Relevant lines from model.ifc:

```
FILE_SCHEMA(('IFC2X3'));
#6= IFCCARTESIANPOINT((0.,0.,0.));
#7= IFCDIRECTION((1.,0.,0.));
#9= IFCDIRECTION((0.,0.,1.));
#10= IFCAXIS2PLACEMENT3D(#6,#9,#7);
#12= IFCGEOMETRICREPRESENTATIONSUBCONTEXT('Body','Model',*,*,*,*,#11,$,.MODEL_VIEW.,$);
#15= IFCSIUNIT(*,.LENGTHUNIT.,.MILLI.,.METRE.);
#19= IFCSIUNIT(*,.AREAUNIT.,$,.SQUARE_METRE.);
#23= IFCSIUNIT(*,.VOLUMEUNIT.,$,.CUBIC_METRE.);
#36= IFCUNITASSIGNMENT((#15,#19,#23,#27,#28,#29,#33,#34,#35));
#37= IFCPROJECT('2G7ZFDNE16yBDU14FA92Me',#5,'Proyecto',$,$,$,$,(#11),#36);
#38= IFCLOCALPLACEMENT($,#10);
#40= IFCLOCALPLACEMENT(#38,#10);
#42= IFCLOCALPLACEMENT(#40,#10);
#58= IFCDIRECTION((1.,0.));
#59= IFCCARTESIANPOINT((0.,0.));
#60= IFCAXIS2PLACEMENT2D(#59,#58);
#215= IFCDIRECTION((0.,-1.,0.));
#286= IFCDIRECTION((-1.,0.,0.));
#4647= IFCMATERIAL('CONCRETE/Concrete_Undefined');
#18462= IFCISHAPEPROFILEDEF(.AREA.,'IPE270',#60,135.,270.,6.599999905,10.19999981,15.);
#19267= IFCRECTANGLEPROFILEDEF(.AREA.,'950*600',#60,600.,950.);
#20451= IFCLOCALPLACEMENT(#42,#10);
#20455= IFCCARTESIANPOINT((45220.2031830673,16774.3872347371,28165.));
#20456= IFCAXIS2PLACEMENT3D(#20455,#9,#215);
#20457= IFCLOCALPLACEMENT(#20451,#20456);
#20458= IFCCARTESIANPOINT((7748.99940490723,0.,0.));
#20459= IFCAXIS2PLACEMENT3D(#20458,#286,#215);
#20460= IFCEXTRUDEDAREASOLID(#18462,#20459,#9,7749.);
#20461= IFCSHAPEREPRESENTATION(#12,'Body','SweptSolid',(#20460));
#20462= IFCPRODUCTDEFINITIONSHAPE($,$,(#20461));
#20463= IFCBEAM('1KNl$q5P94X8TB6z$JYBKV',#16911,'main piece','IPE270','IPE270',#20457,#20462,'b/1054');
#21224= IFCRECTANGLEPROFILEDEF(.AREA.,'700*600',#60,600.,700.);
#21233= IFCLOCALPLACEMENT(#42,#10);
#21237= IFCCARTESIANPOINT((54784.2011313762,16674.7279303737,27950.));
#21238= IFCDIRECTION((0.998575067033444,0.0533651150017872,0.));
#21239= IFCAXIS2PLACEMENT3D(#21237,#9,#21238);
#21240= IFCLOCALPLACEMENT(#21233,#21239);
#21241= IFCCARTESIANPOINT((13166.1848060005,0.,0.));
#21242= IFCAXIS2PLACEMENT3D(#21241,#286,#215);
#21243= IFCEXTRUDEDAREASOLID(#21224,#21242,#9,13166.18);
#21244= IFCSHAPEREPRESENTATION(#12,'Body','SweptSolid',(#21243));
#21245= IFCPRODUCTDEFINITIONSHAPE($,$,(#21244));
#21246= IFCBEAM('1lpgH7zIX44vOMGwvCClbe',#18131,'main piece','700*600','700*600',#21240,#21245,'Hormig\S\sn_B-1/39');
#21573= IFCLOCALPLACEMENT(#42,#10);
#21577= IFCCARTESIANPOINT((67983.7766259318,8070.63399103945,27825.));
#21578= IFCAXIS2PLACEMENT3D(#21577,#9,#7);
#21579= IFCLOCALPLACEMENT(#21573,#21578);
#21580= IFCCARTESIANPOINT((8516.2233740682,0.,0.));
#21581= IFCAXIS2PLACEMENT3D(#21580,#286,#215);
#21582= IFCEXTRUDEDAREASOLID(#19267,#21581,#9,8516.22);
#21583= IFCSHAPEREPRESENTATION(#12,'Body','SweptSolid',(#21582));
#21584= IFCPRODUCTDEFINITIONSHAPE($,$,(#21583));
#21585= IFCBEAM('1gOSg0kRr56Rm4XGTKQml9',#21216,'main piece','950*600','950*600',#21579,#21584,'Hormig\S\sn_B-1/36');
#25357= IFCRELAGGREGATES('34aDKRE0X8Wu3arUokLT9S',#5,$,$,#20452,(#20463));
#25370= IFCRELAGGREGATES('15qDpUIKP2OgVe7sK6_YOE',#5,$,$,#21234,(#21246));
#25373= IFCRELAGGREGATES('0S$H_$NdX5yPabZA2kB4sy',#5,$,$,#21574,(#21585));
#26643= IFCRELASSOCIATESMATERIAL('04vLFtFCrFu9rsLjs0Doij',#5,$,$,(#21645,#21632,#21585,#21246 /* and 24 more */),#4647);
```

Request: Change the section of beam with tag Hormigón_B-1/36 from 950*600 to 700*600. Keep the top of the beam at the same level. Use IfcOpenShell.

```python
import ifcopenshell
import ifcopenshell.util.element
import ifcopenshell.util.representation

model = ifcopenshell.open("model.ifc")

member = model.by_guid("1gOSg0kRr56Rm4XGTKQml9")
source = next(p for p in model.by_type("IfcRectangleProfileDef") if p.ProfileName == "700*600")

body = ifcopenshell.util.representation.get_representation(member, "Model", "Body")
solid = body.Items[0]
old_profile = solid.SweptArea

# Copy the section's sizes but keep this member's own profile position.
profile = ifcopenshell.util.element.copy(model, source)
# Profiles are centred, so shift by half the change in depth to hold the top.
shift = (old_profile.YDim - profile.YDim) / 2
x, y = old_profile.Position.Location.Coordinates
up = (0.0, 1.0)  # upwards, in the solid's own plane
location = model.createIfcCartesianPoint((x + up[0] * shift, y + up[1] * shift))
profile.Position = model.createIfcAxis2Placement2D(location, old_profile.Position.RefDirection)
solid.SweptArea = profile
if not model.get_total_inverses(old_profile):
    ifcopenshell.util.element.remove_deep2(model, old_profile)
member.Description = member.Description.replace("950*600", "700*600")
member.ObjectType = member.ObjectType.replace("950*600", "700*600")

print(solid.SweptArea)

model.write("model-out.ifc")
```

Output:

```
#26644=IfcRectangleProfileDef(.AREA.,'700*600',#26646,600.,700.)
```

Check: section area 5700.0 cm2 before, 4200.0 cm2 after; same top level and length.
